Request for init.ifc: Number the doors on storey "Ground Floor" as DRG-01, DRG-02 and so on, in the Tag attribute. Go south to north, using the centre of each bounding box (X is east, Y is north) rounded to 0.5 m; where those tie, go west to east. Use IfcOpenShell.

First a look at what the model holds.

```python
import ifcopenshell
import ifcopenshell.util.element
import ifcopenshell.util.placement

model = ifcopenshell.open("init.ifc")
print(model.schema)
storey = next(s for s in model.by_type("IfcBuildingStorey") if s.Name == "Ground Floor")
doors = [e for e in ifcopenshell.util.element.get_decomposition(storey) if e.is_a("IfcDoor")]
for e in sorted(doors, key=lambda e: e.id()):
    origin = ifcopenshell.util.placement.get_local_placement(e.ObjectPlacement)[:3, 3]
    print(e.id(), e.Tag, e.Name, origin.round(2) + 0.0, sep=" | ")
```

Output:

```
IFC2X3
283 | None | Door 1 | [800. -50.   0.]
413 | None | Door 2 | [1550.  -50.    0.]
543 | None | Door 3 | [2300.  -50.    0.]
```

```python
import ifcopenshell
import ifcopenshell.geom
import ifcopenshell.util.element
import ifcopenshell.util.shape

model = ifcopenshell.open("init.ifc")
settings = ifcopenshell.geom.settings()
settings.set("use-world-coords", True)


def centre(element):
    shape = ifcopenshell.geom.create_shape(settings, element)
    return ifcopenshell.util.shape.get_bbox_centroid(shape.geometry)


storey = next(s for s in model.by_type("IfcBuildingStorey") if s.Name == "Ground Floor")
doors = [e for e in ifcopenshell.util.element.get_decomposition(storey) if e.is_a("IfcDoor")]

# Insertion points can sit at a corner or the storey origin, so sort by the geometry (in metres).
centres = {e: centre(e) for e in doors}
doors.sort(key=lambda e: (round(centres[e][1] / 0.5), centres[e][0]))

for i, e in enumerate(doors, start=1):
    number = f"DRG-{i:02d}"
    e.Tag = number
    print(e.id(), number)

model.write("init-out.ifc")
```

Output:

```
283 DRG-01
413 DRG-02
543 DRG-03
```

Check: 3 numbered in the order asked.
